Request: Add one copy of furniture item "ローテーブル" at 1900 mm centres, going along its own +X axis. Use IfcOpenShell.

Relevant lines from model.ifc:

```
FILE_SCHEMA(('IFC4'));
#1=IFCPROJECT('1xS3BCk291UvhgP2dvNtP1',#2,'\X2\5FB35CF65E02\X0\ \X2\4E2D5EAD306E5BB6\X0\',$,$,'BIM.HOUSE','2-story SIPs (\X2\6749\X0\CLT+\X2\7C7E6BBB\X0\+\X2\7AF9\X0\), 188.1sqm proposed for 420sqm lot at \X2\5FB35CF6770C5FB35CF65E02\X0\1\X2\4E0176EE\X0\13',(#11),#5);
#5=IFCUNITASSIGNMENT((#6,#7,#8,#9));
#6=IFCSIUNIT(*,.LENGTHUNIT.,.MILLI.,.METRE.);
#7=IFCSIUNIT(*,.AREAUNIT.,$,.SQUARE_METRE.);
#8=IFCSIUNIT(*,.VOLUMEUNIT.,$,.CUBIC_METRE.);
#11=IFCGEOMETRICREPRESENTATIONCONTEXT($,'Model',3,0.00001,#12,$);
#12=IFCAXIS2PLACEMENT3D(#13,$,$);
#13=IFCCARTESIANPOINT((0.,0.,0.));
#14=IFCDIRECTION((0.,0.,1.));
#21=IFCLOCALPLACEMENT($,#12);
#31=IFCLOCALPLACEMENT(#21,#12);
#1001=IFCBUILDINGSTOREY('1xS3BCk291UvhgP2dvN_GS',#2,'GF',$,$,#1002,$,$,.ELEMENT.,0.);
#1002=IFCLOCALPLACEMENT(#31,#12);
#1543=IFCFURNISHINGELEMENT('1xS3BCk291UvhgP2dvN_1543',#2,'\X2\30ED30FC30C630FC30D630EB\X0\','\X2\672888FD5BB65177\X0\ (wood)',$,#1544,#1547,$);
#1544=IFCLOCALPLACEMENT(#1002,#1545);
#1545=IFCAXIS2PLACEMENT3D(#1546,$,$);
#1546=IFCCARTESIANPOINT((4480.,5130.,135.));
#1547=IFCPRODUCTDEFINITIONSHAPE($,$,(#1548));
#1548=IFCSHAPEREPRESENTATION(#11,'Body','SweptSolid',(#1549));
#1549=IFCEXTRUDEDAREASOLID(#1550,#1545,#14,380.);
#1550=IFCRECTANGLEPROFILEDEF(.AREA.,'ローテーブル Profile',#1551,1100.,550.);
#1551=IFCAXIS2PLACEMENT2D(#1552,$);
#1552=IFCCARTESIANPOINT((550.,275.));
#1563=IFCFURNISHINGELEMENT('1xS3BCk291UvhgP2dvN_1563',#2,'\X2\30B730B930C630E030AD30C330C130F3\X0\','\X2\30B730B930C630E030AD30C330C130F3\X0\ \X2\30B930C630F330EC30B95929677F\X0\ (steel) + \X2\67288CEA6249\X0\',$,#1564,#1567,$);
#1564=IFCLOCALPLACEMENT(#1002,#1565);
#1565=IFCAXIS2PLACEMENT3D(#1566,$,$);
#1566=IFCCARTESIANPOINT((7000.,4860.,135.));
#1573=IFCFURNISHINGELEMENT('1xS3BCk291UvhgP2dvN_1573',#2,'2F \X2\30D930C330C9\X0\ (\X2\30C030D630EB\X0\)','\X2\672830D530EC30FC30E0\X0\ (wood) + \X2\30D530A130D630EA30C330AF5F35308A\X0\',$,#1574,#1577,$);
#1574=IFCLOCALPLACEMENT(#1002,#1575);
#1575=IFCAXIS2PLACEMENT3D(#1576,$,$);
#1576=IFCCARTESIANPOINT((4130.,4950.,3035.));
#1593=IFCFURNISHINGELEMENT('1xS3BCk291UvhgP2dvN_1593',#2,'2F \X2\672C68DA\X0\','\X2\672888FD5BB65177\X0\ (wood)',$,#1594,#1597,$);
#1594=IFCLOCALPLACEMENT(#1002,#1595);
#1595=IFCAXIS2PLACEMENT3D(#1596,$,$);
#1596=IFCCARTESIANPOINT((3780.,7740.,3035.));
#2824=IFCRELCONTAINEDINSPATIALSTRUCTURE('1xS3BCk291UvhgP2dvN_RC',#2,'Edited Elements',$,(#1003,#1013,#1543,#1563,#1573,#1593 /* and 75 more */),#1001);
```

```python
import ifcopenshell
import ifcopenshell.api.geometry
import ifcopenshell.api.root
import ifcopenshell.util.element
import ifcopenshell.util.placement
import ifcopenshell.util.unit

model = ifcopenshell.open("model.ifc")
unit_scale = ifcopenshell.util.unit.calculate_unit_scale(model)


def reuse_history(source, copy):
    """copy_class also copies each property set's owner history, people and application; keep the originals."""
    for rel in copy.IsDefinedBy:
        if rel.is_a("IfcRelDefinesByProperties") and (history := rel.RelatingPropertyDefinition.OwnerHistory):
            rel.RelatingPropertyDefinition.OwnerHistory = source.OwnerHistory
            ifcopenshell.util.element.remove_deep2(model, history)


source = model.by_guid("1xS3BCk291UvhgP2dvN_1543")
base = ifcopenshell.util.placement.get_local_placement(source.ObjectPlacement)
step = base[:3, 0] * 1.9 / unit_scale

for i in range(1, 2):
    copy = ifcopenshell.api.root.copy_class(model, product=source)
    copy.Representation = ifcopenshell.util.element.copy_deep(
        model, source.Representation, exclude=["IfcGeometricRepresentationContext", "IfcRepresentationMap"]
    )
    reuse_history(source, copy)
    matrix = base.copy()
    matrix[:3, 3] += i * step
    print("added at", matrix[:3, 3].round(3) + 0.0)
    ifcopenshell.api.geometry.edit_object_placement(model, product=copy, matrix=matrix, is_si=False)

model.write("model_edited.ifc")
```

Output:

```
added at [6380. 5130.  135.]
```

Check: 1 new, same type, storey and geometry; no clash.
